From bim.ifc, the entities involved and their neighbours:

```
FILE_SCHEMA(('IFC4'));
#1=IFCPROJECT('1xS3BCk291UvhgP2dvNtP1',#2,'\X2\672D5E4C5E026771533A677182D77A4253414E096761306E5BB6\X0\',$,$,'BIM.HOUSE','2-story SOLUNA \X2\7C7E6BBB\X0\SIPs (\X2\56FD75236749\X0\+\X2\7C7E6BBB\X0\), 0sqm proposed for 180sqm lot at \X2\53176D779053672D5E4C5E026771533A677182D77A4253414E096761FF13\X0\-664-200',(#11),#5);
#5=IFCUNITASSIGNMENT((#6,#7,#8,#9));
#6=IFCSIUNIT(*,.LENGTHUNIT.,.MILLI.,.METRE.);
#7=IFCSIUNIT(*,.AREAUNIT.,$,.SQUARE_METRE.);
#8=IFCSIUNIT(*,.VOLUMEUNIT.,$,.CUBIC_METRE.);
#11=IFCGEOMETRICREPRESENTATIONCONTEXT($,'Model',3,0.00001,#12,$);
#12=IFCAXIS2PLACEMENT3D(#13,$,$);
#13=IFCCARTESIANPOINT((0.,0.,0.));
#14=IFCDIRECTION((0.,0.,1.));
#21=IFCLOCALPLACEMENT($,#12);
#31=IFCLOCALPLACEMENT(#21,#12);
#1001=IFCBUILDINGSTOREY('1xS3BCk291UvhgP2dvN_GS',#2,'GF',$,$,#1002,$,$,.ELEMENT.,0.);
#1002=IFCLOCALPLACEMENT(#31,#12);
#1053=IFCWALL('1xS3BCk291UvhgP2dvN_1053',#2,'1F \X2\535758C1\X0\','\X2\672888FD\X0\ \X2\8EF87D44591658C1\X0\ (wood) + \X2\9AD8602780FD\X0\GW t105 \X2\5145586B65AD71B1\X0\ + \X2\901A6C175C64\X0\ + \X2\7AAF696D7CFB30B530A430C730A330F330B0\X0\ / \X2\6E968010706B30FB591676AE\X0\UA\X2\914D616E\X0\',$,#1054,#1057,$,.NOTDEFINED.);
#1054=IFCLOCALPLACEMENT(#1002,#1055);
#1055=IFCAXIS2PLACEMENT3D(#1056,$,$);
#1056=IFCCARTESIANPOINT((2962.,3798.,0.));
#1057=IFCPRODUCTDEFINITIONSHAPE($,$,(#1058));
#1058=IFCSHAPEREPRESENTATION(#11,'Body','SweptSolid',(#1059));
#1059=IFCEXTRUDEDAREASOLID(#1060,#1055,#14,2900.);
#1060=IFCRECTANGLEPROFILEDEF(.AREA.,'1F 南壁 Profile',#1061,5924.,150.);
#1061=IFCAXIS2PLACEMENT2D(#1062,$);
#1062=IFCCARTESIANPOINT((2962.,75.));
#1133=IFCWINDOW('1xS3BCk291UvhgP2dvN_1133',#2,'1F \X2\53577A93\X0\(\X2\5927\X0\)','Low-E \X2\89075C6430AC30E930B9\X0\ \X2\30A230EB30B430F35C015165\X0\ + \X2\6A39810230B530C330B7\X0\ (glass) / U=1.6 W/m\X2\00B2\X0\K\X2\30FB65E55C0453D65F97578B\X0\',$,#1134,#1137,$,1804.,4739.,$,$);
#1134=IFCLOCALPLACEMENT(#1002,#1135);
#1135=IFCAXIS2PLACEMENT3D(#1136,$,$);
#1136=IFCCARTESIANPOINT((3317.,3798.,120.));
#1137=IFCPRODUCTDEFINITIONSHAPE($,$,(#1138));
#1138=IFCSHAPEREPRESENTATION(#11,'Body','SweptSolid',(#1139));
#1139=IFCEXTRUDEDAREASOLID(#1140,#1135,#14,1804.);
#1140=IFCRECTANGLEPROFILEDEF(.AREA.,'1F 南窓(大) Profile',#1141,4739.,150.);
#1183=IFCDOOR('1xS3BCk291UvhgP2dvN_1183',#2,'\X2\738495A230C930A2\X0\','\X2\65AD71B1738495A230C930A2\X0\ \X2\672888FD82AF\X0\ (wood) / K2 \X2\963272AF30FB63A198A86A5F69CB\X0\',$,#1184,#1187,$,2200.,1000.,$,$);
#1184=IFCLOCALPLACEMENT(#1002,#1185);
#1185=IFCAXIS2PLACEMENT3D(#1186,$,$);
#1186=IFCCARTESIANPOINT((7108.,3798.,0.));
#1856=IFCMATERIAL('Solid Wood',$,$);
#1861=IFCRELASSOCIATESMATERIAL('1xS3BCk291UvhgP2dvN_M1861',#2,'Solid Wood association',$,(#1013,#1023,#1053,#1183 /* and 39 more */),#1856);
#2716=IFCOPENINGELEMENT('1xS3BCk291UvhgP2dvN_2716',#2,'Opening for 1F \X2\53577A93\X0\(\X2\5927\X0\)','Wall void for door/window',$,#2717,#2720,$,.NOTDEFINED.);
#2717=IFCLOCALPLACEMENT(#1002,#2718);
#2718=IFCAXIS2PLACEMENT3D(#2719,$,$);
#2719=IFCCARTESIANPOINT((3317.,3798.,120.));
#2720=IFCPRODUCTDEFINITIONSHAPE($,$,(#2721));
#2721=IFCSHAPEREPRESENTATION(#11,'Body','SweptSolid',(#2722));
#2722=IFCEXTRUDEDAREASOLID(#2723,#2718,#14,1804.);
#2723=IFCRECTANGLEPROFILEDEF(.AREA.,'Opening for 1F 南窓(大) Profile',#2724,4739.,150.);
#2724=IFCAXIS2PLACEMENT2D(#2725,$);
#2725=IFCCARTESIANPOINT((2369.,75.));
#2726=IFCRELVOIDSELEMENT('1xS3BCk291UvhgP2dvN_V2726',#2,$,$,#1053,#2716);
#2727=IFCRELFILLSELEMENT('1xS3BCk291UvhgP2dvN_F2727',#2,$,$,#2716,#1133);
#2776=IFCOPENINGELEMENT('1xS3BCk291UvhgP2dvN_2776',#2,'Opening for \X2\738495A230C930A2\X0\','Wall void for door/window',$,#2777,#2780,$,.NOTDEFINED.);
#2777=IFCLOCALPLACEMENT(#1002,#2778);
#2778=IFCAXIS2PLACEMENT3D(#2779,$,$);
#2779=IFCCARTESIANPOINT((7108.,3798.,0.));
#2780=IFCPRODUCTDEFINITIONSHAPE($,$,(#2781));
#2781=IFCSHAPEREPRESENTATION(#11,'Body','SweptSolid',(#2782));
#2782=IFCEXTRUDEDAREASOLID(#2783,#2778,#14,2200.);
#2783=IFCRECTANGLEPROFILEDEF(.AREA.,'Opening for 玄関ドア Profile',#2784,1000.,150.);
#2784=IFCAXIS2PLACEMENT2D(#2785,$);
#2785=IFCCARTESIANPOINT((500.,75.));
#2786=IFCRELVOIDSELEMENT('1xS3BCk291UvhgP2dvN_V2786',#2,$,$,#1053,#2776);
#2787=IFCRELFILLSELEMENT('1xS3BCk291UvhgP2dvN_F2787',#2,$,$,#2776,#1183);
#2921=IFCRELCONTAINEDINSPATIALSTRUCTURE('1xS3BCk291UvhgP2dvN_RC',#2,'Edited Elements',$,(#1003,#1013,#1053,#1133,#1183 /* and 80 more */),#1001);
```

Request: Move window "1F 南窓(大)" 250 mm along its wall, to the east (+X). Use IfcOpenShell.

```python
import ifcopenshell
import ifcopenshell.api.geometry
import ifcopenshell.util.placement

model = ifcopenshell.open("bim.ifc")

window = model.by_guid("1xS3BCk291UvhgP2dvN_1133")
opening = window.FillsVoids[0].RelatingOpeningElement
wall = opening.VoidsElements[0].RelatingBuildingElement

wall_matrix = ifcopenshell.util.placement.get_local_placement(wall.ObjectPlacement)
shift = wall_matrix[:3, 0] * 250.0
before = ifcopenshell.util.placement.get_local_placement(window.ObjectPlacement)[:3, 3].copy()

# The window is not placed relative to its opening, so move both.
for product in (opening, window):
    matrix = ifcopenshell.util.placement.get_local_placement(product.ObjectPlacement)
    matrix[:3, 3] += shift
    ifcopenshell.api.geometry.edit_object_placement(model, product=product, matrix=matrix, is_si=False)

after = ifcopenshell.util.placement.get_local_placement(window.ObjectPlacement)[:3, 3]
print("window moved by", (after - before).round(3) + 0.0)

model.write("bim_updated.ifc")
```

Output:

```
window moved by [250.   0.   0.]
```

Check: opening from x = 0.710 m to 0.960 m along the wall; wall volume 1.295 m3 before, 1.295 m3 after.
